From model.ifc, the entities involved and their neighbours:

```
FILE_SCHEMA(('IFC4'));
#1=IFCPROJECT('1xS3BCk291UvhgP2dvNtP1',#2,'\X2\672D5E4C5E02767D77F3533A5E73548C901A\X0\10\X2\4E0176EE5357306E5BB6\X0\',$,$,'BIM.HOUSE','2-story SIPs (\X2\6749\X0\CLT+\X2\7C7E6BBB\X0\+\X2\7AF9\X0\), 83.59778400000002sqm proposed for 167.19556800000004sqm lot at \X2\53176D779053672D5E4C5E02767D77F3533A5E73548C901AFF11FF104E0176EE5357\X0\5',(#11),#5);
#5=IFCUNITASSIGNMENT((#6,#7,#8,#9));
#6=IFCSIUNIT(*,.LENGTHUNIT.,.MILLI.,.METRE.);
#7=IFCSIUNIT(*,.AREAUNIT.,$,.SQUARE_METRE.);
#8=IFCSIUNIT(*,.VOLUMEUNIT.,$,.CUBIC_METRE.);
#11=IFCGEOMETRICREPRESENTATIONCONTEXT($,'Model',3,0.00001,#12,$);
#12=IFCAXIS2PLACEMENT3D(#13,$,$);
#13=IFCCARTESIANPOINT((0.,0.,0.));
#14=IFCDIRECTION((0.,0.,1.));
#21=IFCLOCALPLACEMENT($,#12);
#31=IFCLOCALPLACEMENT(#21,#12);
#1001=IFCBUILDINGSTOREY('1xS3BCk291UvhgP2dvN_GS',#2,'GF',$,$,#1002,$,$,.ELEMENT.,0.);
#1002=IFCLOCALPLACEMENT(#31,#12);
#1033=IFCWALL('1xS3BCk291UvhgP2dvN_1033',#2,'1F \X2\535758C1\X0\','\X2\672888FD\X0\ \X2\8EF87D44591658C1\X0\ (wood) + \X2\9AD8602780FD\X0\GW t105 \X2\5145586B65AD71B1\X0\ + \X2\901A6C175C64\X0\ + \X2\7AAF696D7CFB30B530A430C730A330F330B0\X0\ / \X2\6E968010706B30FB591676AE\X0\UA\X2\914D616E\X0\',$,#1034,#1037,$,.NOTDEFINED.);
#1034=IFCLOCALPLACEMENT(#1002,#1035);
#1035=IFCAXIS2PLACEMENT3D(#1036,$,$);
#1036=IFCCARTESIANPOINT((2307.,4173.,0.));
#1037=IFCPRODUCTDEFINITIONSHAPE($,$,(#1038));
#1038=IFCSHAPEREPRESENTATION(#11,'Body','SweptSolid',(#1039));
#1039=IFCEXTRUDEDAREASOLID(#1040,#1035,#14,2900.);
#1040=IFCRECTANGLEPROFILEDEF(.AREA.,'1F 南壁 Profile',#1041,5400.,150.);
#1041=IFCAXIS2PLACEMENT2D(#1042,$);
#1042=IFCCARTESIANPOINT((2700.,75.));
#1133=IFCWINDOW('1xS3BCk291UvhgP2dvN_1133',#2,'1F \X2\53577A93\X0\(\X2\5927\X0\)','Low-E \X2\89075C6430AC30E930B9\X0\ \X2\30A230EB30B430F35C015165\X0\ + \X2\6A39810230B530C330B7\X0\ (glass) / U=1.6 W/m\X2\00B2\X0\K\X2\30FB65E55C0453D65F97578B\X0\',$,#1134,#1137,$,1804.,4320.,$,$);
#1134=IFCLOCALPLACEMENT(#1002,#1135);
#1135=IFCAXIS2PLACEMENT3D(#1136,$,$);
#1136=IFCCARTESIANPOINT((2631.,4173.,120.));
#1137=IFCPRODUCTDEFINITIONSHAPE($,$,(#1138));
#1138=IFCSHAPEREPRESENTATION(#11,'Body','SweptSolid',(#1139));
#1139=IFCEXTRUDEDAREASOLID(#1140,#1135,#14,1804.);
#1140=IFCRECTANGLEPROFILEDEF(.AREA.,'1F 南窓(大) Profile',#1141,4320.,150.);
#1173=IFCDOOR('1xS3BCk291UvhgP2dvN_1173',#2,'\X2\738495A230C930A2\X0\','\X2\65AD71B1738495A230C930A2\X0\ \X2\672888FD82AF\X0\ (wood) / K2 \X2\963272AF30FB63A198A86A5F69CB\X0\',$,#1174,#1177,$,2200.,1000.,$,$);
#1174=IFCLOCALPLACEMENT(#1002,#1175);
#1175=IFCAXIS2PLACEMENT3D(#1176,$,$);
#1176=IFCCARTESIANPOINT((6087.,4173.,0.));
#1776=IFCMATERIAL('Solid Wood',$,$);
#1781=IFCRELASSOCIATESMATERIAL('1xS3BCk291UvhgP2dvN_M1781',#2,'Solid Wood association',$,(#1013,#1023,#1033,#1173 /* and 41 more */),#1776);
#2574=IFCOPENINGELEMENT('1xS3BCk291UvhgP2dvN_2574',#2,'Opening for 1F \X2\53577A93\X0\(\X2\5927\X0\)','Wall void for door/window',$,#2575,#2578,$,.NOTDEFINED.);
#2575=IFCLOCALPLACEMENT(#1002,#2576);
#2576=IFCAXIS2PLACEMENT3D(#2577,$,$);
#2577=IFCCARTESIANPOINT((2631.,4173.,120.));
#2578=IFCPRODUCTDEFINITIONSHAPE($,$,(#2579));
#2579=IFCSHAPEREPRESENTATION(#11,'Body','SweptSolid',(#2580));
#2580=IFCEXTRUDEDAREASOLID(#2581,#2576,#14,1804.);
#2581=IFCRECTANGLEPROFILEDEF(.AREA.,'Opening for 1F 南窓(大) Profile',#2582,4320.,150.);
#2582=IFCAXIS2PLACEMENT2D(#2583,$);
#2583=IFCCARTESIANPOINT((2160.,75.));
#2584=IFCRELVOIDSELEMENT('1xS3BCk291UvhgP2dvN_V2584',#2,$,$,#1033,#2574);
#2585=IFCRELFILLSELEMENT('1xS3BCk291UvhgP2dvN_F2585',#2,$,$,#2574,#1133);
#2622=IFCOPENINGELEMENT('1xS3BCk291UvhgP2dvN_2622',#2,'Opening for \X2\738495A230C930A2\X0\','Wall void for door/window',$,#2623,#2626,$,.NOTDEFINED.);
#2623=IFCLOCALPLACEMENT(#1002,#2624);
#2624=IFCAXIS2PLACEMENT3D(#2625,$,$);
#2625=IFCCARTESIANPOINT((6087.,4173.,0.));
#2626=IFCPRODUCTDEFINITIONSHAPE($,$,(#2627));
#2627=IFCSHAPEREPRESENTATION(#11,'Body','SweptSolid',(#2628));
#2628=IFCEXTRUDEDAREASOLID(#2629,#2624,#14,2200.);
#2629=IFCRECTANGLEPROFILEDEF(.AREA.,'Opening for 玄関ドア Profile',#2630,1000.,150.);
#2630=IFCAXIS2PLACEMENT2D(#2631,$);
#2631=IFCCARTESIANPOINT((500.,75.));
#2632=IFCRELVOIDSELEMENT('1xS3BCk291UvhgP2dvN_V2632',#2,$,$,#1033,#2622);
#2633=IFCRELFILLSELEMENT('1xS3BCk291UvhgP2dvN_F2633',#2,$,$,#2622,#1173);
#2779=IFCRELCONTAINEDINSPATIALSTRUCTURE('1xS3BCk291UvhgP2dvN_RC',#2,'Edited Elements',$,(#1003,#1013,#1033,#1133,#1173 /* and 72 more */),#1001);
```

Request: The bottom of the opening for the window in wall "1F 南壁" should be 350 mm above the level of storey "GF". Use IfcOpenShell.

```python
import numpy as np
import ifcopenshell
import ifcopenshell.api.geometry
import ifcopenshell.geom
import ifcopenshell.util.element
import ifcopenshell.util.placement
import ifcopenshell.util.shape
import ifcopenshell.util.unit

model = ifcopenshell.open("model.ifc")
unit_scale = ifcopenshell.util.unit.calculate_unit_scale(model)

window = model.by_guid("1xS3BCk291UvhgP2dvN_1133")
opening = window.FillsVoids[0].RelatingOpeningElement
storey = ifcopenshell.util.element.get_container(window, ifc_class="IfcBuildingStorey")
level = ifcopenshell.util.placement.get_local_placement(storey.ObjectPlacement)[2, 3]

# The opening's origin need not be at the sill, so measure its lowest point.
shape = ifcopenshell.geom.create_shape(ifcopenshell.geom.settings(), opening)
bottom = ifcopenshell.util.shape.get_shape_bottom_elevation(shape, shape.geometry) / unit_scale
dz = level + 350.0 - bottom

shift = np.array([0.0, 0.0, dz])
# The window is not placed relative to its opening, so move both.
for product in (opening, window):
    matrix = ifcopenshell.util.placement.get_local_placement(product.ObjectPlacement)
    matrix[:3, 3] += shift
    ifcopenshell.api.geometry.edit_object_placement(model, product=product, matrix=matrix, is_si=False)

print(f"moved by {dz * unit_scale:+.3f} m")

model.write("model_v2.ifc")
```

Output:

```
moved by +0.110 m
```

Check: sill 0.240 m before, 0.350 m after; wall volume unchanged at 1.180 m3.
